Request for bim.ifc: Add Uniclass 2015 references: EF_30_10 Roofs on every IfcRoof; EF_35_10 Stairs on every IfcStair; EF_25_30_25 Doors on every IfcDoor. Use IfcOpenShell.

First a look at what the model holds.

```python
import ifcopenshell

model = ifcopenshell.open("bim.ifc")
print(model.schema)
print("classifications:", [c.Name for c in model.by_type("IfcClassification")])
for ifc_class in ("IfcDoor", "IfcRoof", "IfcStair", "IfcWall", "IfcWindow"):
    print(ifc_class, len(model.by_type(ifc_class)))
```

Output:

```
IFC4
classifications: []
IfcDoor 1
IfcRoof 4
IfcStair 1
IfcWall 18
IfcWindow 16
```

```python
import ifcopenshell
import ifcopenshell.api.classification

model = ifcopenshell.open("bim.ifc")

system = ifcopenshell.api.classification.add_classification(model, classification="Uniclass 2015")

codes = {
    "IfcRoof": ("EF_30_10", "Roofs"),
    "IfcStair": ("EF_35_10", "Stairs"),
    "IfcDoor": ("EF_25_30_25", "Doors"),
}
for ifc_class, (code, name) in codes.items():
    products = model.by_type(ifc_class)
    ifcopenshell.api.classification.add_reference(
        model, products=products, classification=system, identification=code, name=name
    )
    print(code, len(products))

model.write("bim_updated.ifc")
```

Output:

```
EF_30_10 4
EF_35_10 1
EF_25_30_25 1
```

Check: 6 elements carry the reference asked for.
